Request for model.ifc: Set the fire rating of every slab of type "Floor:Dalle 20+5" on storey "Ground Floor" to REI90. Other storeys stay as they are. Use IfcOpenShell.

First a look at what the model holds.

```python
import ifcopenshell
import ifcopenshell.util.element

model = ifcopenshell.open("model.ifc")
print(model.schema)
storey = next(s for s in model.by_type("IfcBuildingStorey") if s.Name == "Ground Floor")
slabs = [e for e in ifcopenshell.util.element.get_decomposition(storey) if e.is_a("IfcSlab")]
seen = {}
for e in slabs:
    element_type = ifcopenshell.util.element.get_type(e)
    key = (element_type.Name if element_type != e and element_type else None, ifcopenshell.util.element.get_pset(e, "Pset_SlabCommon", "FireRating"))
    seen[key] = seen.get(key, 0) + 1
for (name, value), count in sorted(seen.items(), key=str):
    print(count, "x", name, "|", value)
```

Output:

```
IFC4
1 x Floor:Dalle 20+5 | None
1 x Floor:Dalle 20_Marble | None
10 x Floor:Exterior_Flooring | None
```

```python
import ifcopenshell
import ifcopenshell.api.pset
import ifcopenshell.util.element

model = ifcopenshell.open("model.ifc")

storey = next(s for s in model.by_type("IfcBuildingStorey") if s.Name == "Ground Floor")
slabs = [e for e in ifcopenshell.util.element.get_decomposition(storey) if e.is_a("IfcSlab")]

count = 0
for e in slabs:
    element_type = ifcopenshell.util.element.get_type(e)
    if element_type in (None, e) or element_type.Name != "Floor:Dalle 20+5":
        continue
    # add_pset returns the element's existing set when there is one.
    pset = ifcopenshell.api.pset.add_pset(model, product=e, name="Pset_SlabCommon")
    ifcopenshell.api.pset.edit_pset(model, pset=pset, properties={"FireRating": "REI90"})
    count += 1

print(count, "slabs updated")

model.write("model_rev.ifc")
```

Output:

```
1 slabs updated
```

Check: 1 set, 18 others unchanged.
